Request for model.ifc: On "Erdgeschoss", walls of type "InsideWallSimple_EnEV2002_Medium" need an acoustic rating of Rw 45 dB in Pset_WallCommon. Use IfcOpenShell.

First a look at what the model holds.

```python
import ifcopenshell
import ifcopenshell.util.element

model = ifcopenshell.open("model.ifc")
print(model.schema)
storey = next(s for s in model.by_type("IfcBuildingStorey") if s.Name == "Erdgeschoss")
walls = [e for e in ifcopenshell.util.element.get_decomposition(storey) if e.is_a("IfcWall")]
seen = {}
for e in walls:
    element_type = ifcopenshell.util.element.get_type(e)
    key = (element_type.Name if element_type != e and element_type else None, ifcopenshell.util.element.get_pset(e, "Pset_WallCommon", "AcousticRating"))
    seen[key] = seen.get(key, 0) + 1
for (name, value), count in sorted(seen.items(), key=str):
    print(count, "x", name, "|", value)
```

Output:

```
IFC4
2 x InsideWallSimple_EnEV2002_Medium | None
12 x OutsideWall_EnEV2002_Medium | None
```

```python
import ifcopenshell
import ifcopenshell.api.pset
import ifcopenshell.util.element

model = ifcopenshell.open("model.ifc")

storey = next(s for s in model.by_type("IfcBuildingStorey") if s.Name == "Erdgeschoss")
walls = [e for e in ifcopenshell.util.element.get_decomposition(storey) if e.is_a("IfcWall")]

count = 0
for e in walls:
    element_type = ifcopenshell.util.element.get_type(e)
    if element_type in (None, e) or element_type.Name != "InsideWallSimple_EnEV2002_Medium":
        continue
    # add_pset returns the element's existing set when there is one.
    pset = ifcopenshell.api.pset.add_pset(model, product=e, name="Pset_WallCommon")
    ifcopenshell.api.pset.edit_pset(model, pset=pset, properties={"AcousticRating": "Rw 45 dB"})
    count += 1

print(count, "walls updated")

model.write("model-out.ifc")
```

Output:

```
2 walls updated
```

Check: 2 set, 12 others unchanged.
